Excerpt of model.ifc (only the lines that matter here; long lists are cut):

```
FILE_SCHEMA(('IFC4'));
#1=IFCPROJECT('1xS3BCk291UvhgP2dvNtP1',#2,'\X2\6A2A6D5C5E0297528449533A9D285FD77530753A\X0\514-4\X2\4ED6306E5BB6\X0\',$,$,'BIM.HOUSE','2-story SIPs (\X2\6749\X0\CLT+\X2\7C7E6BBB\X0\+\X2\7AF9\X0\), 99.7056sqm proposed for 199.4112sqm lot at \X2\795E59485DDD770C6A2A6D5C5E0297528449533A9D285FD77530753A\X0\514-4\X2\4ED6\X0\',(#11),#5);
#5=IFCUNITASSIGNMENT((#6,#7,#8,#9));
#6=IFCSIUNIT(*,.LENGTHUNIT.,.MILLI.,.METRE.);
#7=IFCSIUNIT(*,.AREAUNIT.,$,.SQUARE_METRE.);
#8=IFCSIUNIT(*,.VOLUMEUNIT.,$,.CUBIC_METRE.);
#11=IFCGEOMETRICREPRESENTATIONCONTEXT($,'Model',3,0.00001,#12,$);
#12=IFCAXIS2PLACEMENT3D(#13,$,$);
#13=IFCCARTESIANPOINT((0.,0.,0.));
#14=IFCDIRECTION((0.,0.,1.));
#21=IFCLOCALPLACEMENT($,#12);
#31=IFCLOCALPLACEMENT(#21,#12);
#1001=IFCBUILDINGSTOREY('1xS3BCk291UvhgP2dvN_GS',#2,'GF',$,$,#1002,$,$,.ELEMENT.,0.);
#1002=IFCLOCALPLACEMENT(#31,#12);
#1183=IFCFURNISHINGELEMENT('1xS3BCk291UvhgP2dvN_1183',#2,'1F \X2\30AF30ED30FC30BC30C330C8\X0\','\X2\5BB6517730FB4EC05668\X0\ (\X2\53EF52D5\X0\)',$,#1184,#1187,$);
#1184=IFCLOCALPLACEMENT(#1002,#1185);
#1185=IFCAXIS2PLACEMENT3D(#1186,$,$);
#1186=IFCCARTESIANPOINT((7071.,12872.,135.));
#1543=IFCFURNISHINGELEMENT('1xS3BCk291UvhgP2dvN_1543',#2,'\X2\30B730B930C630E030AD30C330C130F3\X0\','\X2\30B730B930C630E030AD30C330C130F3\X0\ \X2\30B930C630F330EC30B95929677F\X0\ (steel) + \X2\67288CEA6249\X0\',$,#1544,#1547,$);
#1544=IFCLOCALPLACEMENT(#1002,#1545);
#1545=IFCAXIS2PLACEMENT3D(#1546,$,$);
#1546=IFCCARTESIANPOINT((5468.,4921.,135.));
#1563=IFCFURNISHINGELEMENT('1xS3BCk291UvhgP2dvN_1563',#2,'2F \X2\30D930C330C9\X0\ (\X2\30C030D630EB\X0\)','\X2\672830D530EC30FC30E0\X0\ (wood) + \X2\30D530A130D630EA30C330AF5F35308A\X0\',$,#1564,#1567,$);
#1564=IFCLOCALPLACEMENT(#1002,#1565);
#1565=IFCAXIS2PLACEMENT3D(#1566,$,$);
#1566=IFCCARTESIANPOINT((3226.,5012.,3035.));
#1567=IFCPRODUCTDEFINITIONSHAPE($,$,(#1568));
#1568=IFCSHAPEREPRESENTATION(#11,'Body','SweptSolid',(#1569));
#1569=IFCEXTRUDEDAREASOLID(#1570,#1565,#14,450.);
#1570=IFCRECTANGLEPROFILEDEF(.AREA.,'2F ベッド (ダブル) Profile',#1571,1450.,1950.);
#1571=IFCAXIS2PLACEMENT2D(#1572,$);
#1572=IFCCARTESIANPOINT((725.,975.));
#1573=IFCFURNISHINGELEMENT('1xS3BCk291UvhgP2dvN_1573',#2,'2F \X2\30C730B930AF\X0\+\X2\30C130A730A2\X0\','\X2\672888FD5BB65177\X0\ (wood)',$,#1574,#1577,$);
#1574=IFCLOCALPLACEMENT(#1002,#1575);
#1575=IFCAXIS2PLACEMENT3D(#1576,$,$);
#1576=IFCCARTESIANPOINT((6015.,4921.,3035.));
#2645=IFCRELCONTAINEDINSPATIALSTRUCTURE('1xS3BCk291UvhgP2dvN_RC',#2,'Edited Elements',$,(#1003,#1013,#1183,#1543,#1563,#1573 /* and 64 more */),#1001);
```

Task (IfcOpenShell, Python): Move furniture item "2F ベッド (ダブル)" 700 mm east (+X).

```python
import ifcopenshell
import ifcopenshell.api.geometry
import ifcopenshell.util.placement

model = ifcopenshell.open("model.ifc")

item = model.by_guid("1xS3BCk291UvhgP2dvN_1563")
matrix = ifcopenshell.util.placement.get_local_placement(item.ObjectPlacement)
matrix[0, 3] += 700.0
ifcopenshell.api.geometry.edit_object_placement(model, product=item, matrix=matrix, is_si=False)

print(ifcopenshell.util.placement.get_local_placement(item.ObjectPlacement).round(3) + 0.0)

model.write("model_rev.ifc")
```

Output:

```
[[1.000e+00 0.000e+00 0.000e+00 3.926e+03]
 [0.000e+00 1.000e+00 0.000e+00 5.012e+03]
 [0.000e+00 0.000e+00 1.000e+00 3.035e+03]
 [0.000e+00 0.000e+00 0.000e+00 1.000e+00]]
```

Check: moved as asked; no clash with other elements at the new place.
